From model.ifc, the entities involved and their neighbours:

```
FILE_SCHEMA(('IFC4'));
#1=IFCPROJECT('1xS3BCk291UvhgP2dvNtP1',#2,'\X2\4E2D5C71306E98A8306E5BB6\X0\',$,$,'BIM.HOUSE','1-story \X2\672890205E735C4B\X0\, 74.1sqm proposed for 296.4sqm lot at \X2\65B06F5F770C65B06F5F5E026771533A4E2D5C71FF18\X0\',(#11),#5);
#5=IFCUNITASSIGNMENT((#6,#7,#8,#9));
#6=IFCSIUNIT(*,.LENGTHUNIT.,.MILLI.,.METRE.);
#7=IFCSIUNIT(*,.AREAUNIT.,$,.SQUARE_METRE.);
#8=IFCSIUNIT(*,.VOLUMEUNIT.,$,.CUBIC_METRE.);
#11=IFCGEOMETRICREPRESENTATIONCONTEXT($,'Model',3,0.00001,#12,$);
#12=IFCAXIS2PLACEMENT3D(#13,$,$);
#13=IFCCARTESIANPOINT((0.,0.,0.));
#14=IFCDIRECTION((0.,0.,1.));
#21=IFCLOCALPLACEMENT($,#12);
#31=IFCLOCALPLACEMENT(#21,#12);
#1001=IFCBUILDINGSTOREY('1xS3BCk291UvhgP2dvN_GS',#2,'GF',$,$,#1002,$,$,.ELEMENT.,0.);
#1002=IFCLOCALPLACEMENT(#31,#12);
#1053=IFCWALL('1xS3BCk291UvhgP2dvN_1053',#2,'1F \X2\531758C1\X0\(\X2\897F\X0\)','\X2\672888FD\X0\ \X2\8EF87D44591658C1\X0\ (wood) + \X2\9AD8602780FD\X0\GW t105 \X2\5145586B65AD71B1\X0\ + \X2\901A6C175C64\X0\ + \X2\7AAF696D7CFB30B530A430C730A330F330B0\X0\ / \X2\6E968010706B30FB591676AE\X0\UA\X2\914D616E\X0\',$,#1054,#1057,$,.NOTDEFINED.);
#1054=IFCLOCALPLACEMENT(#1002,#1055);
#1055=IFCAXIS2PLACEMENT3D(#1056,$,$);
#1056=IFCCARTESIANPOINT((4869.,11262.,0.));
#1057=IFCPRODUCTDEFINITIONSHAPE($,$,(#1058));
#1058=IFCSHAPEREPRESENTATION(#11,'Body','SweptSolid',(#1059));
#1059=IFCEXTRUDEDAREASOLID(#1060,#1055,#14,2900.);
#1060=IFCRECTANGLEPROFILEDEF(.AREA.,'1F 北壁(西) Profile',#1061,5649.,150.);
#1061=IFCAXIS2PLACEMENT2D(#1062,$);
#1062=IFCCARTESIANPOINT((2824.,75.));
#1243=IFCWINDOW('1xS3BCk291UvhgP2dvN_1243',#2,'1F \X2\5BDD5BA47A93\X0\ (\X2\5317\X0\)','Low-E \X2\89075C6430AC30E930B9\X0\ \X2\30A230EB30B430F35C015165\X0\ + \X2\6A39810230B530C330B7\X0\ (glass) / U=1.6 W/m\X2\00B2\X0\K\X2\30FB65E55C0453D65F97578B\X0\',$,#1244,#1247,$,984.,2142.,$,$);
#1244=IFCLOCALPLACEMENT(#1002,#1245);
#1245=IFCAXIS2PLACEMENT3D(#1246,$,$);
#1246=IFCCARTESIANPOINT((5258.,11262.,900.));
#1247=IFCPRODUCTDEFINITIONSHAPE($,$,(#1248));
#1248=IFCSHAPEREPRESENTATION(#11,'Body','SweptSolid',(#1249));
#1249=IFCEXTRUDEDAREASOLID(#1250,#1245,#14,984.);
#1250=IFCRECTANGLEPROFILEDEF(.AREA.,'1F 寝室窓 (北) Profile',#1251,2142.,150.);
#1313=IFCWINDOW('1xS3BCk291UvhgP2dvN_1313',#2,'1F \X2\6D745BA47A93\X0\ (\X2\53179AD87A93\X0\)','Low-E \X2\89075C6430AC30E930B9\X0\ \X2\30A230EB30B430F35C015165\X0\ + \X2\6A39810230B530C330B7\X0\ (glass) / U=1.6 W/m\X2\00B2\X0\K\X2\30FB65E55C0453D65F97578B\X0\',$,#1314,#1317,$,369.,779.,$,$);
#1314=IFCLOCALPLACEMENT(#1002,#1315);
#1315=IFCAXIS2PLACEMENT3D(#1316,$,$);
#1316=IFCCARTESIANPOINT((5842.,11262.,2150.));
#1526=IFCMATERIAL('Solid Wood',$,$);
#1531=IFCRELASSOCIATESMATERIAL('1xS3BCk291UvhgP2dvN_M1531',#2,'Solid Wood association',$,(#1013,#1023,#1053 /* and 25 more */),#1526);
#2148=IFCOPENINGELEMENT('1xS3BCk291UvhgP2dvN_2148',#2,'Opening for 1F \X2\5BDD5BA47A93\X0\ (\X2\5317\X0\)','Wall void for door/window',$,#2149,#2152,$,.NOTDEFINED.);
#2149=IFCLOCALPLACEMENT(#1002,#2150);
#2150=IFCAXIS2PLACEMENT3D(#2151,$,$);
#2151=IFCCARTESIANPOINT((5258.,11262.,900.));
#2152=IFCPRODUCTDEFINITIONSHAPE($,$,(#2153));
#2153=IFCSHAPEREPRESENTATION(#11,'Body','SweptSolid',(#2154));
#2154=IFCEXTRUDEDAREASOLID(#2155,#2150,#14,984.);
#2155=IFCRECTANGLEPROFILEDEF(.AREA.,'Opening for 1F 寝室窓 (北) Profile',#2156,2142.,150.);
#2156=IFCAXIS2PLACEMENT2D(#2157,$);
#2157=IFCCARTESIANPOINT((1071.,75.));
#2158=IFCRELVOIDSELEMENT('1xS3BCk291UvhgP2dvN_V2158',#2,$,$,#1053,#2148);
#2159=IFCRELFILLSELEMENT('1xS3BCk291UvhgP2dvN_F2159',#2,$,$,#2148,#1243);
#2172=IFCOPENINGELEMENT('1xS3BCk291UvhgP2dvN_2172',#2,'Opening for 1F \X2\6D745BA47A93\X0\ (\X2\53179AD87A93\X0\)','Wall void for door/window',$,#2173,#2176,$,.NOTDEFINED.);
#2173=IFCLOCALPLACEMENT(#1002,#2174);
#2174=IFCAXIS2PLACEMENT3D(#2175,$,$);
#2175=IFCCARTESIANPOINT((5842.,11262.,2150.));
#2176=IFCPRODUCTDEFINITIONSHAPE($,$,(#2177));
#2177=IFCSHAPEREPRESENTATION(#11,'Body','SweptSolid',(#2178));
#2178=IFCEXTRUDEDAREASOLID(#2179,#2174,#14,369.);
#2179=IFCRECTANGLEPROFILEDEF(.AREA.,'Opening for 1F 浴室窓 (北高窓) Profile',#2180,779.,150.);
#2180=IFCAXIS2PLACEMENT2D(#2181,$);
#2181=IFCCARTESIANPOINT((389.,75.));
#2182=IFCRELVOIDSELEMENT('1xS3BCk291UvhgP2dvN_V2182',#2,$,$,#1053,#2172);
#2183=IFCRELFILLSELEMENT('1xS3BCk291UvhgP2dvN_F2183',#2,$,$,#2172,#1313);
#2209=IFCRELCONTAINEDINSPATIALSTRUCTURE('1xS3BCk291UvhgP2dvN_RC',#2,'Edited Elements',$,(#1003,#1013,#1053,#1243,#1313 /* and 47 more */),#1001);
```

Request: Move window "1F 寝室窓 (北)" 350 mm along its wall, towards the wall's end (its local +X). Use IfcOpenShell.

```python
import ifcopenshell
import ifcopenshell.api.geometry
import ifcopenshell.util.placement

model = ifcopenshell.open("model.ifc")

window = model.by_guid("1xS3BCk291UvhgP2dvN_1243")
opening = window.FillsVoids[0].RelatingOpeningElement
wall = opening.VoidsElements[0].RelatingBuildingElement

wall_matrix = ifcopenshell.util.placement.get_local_placement(wall.ObjectPlacement)
shift = wall_matrix[:3, 0] * 350.0
before = ifcopenshell.util.placement.get_local_placement(window.ObjectPlacement)[:3, 3].copy()

# The window is not placed relative to its opening, so move both.
for product in (opening, window):
    matrix = ifcopenshell.util.placement.get_local_placement(product.ObjectPlacement)
    matrix[:3, 3] += shift
    ifcopenshell.api.geometry.edit_object_placement(model, product=product, matrix=matrix, is_si=False)

after = ifcopenshell.util.placement.get_local_placement(window.ObjectPlacement)[:3, 3]
print("window moved by", (after - before).round(3) + 0.0)

model.write("model_updated.ifc")
```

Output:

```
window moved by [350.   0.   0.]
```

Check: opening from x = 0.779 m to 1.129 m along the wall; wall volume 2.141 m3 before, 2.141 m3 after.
